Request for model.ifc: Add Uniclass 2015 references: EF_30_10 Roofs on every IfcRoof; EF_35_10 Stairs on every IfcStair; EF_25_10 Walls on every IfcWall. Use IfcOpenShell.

First a look at what the model holds.

```python
import ifcopenshell

model = ifcopenshell.open("model.ifc")
print(model.schema)
print("classifications:", [c.Name for c in model.by_type("IfcClassification")])
for ifc_class in ("IfcDoor", "IfcRoof", "IfcStair", "IfcWall", "IfcWindow"):
    print(ifc_class, len(model.by_type(ifc_class)))
```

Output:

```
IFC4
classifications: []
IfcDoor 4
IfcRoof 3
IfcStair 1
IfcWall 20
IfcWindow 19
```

```python
import ifcopenshell
import ifcopenshell.api.classification

model = ifcopenshell.open("model.ifc")

system = ifcopenshell.api.classification.add_classification(model, classification="Uniclass 2015")

codes = {
    "IfcRoof": ("EF_30_10", "Roofs"),
    "IfcStair": ("EF_35_10", "Stairs"),
    "IfcWall": ("EF_25_10", "Walls"),
}
for ifc_class, (code, name) in codes.items():
    products = model.by_type(ifc_class)
    ifcopenshell.api.classification.add_reference(
        model, products=products, classification=system, identification=code, name=name
    )
    print(code, len(products))

model.write("model_v2.ifc")
```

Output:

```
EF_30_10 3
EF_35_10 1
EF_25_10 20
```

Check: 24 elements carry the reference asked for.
